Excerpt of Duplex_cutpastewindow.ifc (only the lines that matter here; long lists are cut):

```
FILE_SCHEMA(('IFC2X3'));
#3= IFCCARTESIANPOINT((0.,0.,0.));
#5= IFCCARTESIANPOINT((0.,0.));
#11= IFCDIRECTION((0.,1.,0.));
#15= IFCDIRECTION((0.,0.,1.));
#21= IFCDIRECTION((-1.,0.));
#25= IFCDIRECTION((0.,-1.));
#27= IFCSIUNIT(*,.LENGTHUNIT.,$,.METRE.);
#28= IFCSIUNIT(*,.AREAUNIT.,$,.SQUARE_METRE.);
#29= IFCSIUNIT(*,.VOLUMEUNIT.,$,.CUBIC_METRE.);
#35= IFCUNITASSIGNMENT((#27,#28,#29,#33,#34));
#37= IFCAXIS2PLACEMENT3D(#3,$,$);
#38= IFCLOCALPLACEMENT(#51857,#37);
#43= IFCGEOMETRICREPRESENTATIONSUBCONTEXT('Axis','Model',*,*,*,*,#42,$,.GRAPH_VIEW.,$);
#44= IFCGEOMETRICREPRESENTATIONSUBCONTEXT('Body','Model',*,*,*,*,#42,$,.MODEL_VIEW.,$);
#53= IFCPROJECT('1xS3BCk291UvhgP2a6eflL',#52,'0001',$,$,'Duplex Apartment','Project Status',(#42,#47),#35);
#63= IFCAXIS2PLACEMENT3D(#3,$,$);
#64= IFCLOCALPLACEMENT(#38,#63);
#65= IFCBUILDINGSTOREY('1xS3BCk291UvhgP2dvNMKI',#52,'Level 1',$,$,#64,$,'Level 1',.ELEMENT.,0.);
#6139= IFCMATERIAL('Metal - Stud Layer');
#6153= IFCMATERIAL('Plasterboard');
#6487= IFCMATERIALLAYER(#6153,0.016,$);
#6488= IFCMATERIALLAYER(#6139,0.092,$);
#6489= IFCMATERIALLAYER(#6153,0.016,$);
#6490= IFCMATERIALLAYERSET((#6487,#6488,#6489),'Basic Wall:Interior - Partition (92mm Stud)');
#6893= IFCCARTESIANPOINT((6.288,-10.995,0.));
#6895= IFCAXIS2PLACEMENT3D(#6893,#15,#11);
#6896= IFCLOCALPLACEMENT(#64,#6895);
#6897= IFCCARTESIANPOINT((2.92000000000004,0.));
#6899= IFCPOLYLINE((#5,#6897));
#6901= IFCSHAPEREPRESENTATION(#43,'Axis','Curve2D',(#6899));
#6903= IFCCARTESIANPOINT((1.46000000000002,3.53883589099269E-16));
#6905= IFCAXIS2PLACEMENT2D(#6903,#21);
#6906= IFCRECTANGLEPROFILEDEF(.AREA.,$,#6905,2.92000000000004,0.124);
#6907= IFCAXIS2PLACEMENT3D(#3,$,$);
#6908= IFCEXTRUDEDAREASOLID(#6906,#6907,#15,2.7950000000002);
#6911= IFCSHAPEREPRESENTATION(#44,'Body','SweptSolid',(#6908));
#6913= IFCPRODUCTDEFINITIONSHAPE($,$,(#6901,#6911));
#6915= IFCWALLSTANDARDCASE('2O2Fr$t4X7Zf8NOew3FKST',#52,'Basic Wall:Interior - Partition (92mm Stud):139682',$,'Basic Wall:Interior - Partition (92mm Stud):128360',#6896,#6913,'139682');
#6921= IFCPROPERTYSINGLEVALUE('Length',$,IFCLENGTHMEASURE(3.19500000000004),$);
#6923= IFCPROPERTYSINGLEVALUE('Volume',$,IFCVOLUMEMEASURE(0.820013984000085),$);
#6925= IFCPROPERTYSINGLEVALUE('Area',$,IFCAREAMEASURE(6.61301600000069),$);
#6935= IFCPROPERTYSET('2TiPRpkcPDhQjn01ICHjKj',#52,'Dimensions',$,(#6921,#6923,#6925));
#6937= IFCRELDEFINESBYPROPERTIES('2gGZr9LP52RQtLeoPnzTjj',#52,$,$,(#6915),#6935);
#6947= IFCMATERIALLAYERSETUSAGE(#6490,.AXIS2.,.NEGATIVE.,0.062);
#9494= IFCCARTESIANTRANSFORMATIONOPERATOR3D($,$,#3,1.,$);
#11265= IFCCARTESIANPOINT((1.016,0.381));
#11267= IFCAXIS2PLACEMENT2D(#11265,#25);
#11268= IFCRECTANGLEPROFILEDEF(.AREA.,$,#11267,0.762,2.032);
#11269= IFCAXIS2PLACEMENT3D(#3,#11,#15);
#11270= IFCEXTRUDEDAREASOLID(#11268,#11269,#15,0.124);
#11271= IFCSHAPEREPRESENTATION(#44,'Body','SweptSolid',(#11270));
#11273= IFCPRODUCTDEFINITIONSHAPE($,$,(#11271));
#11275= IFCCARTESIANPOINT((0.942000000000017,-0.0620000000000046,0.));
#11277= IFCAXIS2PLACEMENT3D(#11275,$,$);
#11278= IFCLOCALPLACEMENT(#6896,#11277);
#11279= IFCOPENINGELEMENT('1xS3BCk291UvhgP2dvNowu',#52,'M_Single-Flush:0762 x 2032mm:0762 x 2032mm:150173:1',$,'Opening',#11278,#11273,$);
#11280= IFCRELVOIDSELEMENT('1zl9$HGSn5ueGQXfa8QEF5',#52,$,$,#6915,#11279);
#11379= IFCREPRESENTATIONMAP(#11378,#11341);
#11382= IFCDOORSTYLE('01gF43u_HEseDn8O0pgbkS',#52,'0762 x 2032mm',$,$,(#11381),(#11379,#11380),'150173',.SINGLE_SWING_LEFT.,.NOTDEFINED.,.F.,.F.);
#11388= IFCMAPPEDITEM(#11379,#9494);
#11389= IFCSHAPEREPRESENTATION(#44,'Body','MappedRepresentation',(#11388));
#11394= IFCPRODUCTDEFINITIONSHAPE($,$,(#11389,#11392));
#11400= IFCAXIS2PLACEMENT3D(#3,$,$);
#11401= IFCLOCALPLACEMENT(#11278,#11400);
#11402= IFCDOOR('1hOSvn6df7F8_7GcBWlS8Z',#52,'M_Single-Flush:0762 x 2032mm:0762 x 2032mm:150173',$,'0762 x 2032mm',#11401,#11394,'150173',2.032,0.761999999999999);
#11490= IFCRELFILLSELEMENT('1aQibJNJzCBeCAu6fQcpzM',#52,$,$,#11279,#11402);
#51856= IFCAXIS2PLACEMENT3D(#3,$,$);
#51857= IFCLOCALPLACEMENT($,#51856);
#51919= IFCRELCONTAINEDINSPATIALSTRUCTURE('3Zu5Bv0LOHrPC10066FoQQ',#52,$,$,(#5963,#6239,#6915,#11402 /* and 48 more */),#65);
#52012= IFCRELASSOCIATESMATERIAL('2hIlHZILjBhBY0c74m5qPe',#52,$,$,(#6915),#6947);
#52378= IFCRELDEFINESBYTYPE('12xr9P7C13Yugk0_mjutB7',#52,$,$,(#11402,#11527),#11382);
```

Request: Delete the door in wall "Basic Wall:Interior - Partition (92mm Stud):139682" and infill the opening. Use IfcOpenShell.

```python
import ifcopenshell
import ifcopenshell.api.feature
import ifcopenshell.api.pset
import ifcopenshell.api.root
import ifcopenshell.geom
import ifcopenshell.util.element
import ifcopenshell.util.shape
import ifcopenshell.util.unit

model = ifcopenshell.open("Duplex_cutpastewindow.ifc")
area_scale = ifcopenshell.util.unit.calculate_unit_scale(model, "AREAUNIT")
volume_scale = ifcopenshell.util.unit.calculate_unit_scale(model, "VOLUMEUNIT")
settings = ifcopenshell.geom.settings()


def volume(element):
    """Net volume in cubic metres, openings subtracted."""
    shape = ifcopenshell.geom.create_shape(settings, element)
    return ifcopenshell.util.shape.get_volume(shape.geometry)


door = model.by_guid("1hOSvn6df7F8_7GcBWlS8Z")
opening = door.FillsVoids[0].RelatingOpeningElement
wall = opening.VoidsElements[0].RelatingBuildingElement
before = volume(wall)

ifcopenshell.api.root.remove_product(model, product=door)
ifcopenshell.api.feature.remove_feature(model, feature=opening)

after = volume(wall)
thickness = 0.124  # wall thickness in metres

# Update the wall's stored quantities.
pset = model.by_id(ifcopenshell.util.element.get_pset(wall, "Dimensions", should_inherit=False)["id"])
ifcopenshell.api.pset.edit_pset(model, pset=pset, properties={
    "Volume": model.create_entity("IfcVolumeMeasure", after / volume_scale),
    "Area": model.create_entity("IfcAreaMeasure", after / thickness / area_scale),
})

print(f"wall volume {before:.3f} -> {after:.3f} m3")

model.write("Duplex_cutpastewindow_v2.ifc")
```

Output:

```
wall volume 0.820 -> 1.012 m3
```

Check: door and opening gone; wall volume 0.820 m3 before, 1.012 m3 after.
